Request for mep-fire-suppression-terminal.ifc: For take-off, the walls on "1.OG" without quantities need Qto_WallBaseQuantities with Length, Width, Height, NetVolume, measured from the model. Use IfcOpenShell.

First a look at what the model holds.

```python
import ifcopenshell
import ifcopenshell.util.element
import ifcopenshell.util.unit

model = ifcopenshell.open("mep-fire-suppression-terminal.ifc")
print(model.schema)
for unit_type in ("LENGTHUNIT", "AREAUNIT", "VOLUMEUNIT"):
    print(unit_type, ifcopenshell.util.unit.calculate_unit_scale(model, unit_type))
storey = next(s for s in model.by_type("IfcBuildingStorey") if s.Name == "1.OG")
walls = [e for e in ifcopenshell.util.element.get_decomposition(storey) if e.is_a("IfcWall")]
for e in sorted(walls, key=lambda e: e.id()):
    print(e.id(), e.is_a(), e.Name, list(ifcopenshell.util.element.get_psets(e, qtos_only=True)), sep=" | ")
```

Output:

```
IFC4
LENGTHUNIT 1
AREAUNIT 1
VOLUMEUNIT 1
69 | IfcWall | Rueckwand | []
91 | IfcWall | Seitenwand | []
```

```python
import ifcopenshell
import ifcopenshell.api.pset
import ifcopenshell.geom
import ifcopenshell.util.element
import ifcopenshell.util.shape
import ifcopenshell.util.unit

model = ifcopenshell.open("mep-fire-suppression-terminal.ifc")
unit_scale = ifcopenshell.util.unit.calculate_unit_scale(model)
volume_scale = ifcopenshell.util.unit.calculate_unit_scale(model, "VOLUMEUNIT")
settings = ifcopenshell.geom.settings()

storey = next(s for s in model.by_type("IfcBuildingStorey") if s.Name == "1.OG")
walls = [e for e in ifcopenshell.util.element.get_decomposition(storey) if e.is_a("IfcWall")]

for e in sorted(walls, key=lambda e: e.id()):
    if ifcopenshell.util.element.get_psets(e, qtos_only=True, should_inherit=False):
        continue
    # Geometry comes back in metres, in the element's own axes.
    shape = ifcopenshell.geom.create_shape(settings, e)
    values = {
        "Length": ifcopenshell.util.shape.get_x(shape.geometry) / unit_scale,
        "Width": ifcopenshell.util.shape.get_y(shape.geometry) / unit_scale,
        "Height": ifcopenshell.util.shape.get_z(shape.geometry) / unit_scale,
        "NetVolume": ifcopenshell.util.shape.get_volume(shape.geometry) / volume_scale,
    }
    qto = ifcopenshell.api.pset.add_qto(model, product=e, name="Qto_WallBaseQuantities")
    ifcopenshell.api.pset.edit_qto(model, qto=qto, properties=values)
    print(e.id(), {k: round(v, 3) for k, v in values.items()})

model.write("mep-fire-suppression-terminal_edited.ifc")
```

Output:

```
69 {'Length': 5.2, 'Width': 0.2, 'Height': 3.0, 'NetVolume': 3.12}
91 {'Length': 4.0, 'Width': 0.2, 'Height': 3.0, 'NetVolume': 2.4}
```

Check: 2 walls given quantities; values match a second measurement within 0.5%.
